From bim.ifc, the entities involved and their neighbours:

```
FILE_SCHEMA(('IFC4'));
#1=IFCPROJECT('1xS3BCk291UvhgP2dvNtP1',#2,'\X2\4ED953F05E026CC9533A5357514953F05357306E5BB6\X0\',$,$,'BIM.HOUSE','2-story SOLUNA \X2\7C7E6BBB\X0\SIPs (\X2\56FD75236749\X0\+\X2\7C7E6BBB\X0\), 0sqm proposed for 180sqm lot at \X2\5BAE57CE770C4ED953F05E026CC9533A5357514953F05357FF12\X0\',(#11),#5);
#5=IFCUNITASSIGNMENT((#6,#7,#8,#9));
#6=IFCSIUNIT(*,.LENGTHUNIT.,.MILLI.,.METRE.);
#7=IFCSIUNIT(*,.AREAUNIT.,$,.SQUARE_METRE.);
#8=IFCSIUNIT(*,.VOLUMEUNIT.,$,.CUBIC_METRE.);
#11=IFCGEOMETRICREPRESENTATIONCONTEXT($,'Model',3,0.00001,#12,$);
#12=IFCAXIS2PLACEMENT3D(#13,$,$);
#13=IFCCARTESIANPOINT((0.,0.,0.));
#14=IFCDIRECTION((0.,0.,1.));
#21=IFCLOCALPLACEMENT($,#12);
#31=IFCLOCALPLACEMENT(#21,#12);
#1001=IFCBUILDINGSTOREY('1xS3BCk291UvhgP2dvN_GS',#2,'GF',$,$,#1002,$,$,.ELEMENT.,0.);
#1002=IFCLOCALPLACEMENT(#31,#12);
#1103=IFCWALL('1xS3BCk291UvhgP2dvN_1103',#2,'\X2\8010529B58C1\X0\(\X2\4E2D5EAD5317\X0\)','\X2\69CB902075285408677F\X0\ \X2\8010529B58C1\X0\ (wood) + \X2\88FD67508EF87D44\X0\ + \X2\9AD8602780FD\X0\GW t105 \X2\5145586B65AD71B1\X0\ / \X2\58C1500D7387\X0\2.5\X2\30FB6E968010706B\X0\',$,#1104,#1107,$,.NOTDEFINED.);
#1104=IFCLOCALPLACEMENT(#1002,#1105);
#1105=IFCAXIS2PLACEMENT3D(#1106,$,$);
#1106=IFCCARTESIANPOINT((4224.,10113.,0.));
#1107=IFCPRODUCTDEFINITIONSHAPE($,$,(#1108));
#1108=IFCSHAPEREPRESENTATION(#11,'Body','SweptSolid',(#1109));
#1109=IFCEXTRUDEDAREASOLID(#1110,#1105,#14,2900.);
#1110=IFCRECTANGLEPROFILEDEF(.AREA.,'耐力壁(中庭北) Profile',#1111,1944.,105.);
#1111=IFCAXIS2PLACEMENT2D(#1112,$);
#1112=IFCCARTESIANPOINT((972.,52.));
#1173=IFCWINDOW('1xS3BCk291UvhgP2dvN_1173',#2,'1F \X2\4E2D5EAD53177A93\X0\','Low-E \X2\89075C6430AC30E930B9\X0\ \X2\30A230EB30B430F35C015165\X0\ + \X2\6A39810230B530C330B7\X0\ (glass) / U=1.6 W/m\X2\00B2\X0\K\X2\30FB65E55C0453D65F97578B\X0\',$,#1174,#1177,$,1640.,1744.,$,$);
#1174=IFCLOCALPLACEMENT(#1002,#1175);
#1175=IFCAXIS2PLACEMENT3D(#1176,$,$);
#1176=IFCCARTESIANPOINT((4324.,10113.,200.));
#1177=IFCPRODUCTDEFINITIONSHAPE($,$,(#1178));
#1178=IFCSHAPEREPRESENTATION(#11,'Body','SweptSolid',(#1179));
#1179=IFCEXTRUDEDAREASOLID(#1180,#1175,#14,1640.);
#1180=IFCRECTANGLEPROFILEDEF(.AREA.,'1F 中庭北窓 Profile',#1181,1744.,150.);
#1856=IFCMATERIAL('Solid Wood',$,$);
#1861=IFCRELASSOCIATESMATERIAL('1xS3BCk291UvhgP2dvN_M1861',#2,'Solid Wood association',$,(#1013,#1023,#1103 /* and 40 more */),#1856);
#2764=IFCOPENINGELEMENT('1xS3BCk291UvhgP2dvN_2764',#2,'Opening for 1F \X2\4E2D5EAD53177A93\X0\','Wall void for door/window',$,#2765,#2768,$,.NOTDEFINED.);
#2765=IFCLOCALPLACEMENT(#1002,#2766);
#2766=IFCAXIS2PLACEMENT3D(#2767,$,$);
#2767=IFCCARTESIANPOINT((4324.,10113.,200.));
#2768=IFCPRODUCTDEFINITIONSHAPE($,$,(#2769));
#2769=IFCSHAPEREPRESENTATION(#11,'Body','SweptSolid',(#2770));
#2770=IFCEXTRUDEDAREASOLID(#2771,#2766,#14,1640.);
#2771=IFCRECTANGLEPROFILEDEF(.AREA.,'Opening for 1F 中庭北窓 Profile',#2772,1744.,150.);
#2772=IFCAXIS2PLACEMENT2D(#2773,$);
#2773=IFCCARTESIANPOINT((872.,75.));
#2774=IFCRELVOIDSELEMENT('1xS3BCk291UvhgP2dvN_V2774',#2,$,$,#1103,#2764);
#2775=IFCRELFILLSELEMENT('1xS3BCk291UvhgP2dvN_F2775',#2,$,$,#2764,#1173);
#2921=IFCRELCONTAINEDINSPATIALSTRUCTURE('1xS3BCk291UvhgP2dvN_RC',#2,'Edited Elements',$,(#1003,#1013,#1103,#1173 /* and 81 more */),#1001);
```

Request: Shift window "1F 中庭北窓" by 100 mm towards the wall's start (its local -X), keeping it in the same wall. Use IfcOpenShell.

```python
import ifcopenshell
import ifcopenshell.api.geometry
import ifcopenshell.util.placement
import ifcopenshell.util.unit

model = ifcopenshell.open("bim.ifc")
unit_scale = ifcopenshell.util.unit.calculate_unit_scale(model)

window = model.by_guid("1xS3BCk291UvhgP2dvN_1173")
opening = window.FillsVoids[0].RelatingOpeningElement
wall = opening.VoidsElements[0].RelatingBuildingElement

wall_matrix = ifcopenshell.util.placement.get_local_placement(wall.ObjectPlacement)
shift = wall_matrix[:3, 0] * -0.1 / unit_scale
before = ifcopenshell.util.placement.get_local_placement(window.ObjectPlacement)[:3, 3].copy()

# The window is not placed relative to its opening, so move both.
for product in (opening, window):
    matrix = ifcopenshell.util.placement.get_local_placement(product.ObjectPlacement)
    matrix[:3, 3] += shift
    ifcopenshell.api.geometry.edit_object_placement(model, product=product, matrix=matrix, is_si=False)

after = ifcopenshell.util.placement.get_local_placement(window.ObjectPlacement)[:3, 3]
print("window moved by", (after - before).round(3) + 0.0)

model.write("bim_rev.ifc")
```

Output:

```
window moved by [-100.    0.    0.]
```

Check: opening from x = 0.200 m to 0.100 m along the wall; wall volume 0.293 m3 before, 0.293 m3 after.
